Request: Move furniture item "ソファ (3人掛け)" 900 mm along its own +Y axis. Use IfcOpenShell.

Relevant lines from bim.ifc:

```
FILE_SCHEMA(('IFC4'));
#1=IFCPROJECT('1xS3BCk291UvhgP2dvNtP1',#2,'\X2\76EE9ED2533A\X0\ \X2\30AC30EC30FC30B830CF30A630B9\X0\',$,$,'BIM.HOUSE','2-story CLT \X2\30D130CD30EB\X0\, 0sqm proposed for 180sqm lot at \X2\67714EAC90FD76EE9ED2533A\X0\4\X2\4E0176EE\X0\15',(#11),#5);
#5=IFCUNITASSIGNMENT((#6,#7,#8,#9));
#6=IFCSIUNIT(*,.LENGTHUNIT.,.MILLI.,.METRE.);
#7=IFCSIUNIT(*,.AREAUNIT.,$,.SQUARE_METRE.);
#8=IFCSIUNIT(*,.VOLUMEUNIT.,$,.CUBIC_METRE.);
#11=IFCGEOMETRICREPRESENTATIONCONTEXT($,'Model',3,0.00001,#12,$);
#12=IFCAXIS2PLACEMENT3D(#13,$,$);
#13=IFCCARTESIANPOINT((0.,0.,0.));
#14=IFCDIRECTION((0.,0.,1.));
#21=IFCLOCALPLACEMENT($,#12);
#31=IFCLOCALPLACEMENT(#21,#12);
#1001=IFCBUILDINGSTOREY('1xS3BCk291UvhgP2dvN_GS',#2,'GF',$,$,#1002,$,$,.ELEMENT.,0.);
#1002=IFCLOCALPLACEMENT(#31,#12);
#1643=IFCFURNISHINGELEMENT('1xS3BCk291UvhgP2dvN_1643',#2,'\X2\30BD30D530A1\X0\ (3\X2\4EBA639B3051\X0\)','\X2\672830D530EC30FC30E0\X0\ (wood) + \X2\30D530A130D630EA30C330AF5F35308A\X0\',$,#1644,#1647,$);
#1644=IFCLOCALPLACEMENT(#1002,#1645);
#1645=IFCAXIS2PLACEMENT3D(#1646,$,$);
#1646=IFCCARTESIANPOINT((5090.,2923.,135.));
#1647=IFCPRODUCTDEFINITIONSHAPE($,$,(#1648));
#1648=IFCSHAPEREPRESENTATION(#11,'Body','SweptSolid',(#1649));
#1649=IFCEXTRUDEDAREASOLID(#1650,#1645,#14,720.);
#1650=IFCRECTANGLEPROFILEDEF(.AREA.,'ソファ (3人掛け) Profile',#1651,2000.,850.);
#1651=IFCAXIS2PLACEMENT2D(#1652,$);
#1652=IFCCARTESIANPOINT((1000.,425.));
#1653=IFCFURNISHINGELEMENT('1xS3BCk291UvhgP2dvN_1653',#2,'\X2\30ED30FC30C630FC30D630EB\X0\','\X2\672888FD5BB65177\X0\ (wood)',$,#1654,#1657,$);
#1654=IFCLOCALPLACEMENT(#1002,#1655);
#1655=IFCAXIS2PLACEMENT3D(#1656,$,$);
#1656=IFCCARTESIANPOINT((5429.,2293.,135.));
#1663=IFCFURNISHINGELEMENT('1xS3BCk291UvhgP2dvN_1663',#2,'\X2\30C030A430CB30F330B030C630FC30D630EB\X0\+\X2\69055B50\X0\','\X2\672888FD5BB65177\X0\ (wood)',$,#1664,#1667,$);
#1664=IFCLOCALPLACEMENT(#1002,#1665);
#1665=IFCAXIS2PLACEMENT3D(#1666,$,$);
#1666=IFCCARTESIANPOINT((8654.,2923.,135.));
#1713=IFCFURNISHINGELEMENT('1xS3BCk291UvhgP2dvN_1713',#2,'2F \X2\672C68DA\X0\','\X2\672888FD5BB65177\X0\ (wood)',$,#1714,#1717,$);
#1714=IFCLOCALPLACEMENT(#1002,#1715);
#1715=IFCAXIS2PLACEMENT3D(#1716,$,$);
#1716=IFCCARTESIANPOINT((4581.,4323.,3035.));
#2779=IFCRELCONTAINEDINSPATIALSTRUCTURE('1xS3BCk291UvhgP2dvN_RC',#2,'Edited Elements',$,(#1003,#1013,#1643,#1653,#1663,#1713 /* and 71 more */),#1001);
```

```python
import ifcopenshell
import ifcopenshell.api.geometry
import ifcopenshell.util.placement
import ifcopenshell.util.unit

model = ifcopenshell.open("bim.ifc")
unit_scale = ifcopenshell.util.unit.calculate_unit_scale(model)

item = model.by_guid("1xS3BCk291UvhgP2dvN_1643")
matrix = ifcopenshell.util.placement.get_local_placement(item.ObjectPlacement)
matrix[:3, 3] += matrix[:3, 1] * 0.9 / unit_scale
ifcopenshell.api.geometry.edit_object_placement(model, product=item, matrix=matrix, is_si=False)

print(ifcopenshell.util.placement.get_local_placement(item.ObjectPlacement).round(3) + 0.0)

model.write("bim_rev.ifc")
```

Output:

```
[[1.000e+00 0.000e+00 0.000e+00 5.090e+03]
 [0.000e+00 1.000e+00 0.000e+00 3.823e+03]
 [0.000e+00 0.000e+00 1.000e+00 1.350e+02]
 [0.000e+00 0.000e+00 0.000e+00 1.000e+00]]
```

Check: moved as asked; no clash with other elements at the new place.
